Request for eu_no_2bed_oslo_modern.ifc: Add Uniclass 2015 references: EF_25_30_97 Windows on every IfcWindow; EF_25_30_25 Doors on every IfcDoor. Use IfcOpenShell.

First a look at what the model holds.

```python
import ifcopenshell

model = ifcopenshell.open("eu_no_2bed_oslo_modern.ifc")
print(model.schema)
print("classifications:", [c.Name for c in model.by_type("IfcClassification")])
for ifc_class in ("IfcDoor", "IfcRoof", "IfcStair", "IfcWall", "IfcWindow"):
    print(ifc_class, len(model.by_type(ifc_class)))
```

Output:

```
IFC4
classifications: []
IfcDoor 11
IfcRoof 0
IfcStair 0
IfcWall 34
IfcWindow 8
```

```python
import ifcopenshell
import ifcopenshell.api.classification

model = ifcopenshell.open("eu_no_2bed_oslo_modern.ifc")

system = ifcopenshell.api.classification.add_classification(model, classification="Uniclass 2015")

codes = {
    "IfcWindow": ("EF_25_30_97", "Windows"),
    "IfcDoor": ("EF_25_30_25", "Doors"),
}
for ifc_class, (code, name) in codes.items():
    products = model.by_type(ifc_class)
    ifcopenshell.api.classification.add_reference(
        model, products=products, classification=system, identification=code, name=name
    )
    print(code, len(products))

model.write("eu_no_2bed_oslo_modern_updated.ifc")
```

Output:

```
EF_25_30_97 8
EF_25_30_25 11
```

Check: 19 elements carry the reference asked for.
